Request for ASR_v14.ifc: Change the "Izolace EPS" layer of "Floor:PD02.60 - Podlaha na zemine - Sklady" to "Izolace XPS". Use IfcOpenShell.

First a look at what the model holds.

```python
import ifcopenshell
import ifcopenshell.util.element

model = ifcopenshell.open("ASR_v14.ifc")
print(model.schema)
for layer_set in model.by_type("IfcMaterialLayerSet"):
    if layer_set.LayerSetName == "Floor:PD02.60 - Podlaha na zemine - Sklady":
        for layer in layer_set.MaterialLayers:
            print(layer.id(), layer.Material and layer.Material.Name, layer.LayerThickness, sep=" | ")
        print(len(ifcopenshell.util.element.get_elements_by_material(model, layer_set)), "elements and types use it")
print(sorted(m.Name for m in model.by_type("IfcMaterial") if m.Name)[:60])
```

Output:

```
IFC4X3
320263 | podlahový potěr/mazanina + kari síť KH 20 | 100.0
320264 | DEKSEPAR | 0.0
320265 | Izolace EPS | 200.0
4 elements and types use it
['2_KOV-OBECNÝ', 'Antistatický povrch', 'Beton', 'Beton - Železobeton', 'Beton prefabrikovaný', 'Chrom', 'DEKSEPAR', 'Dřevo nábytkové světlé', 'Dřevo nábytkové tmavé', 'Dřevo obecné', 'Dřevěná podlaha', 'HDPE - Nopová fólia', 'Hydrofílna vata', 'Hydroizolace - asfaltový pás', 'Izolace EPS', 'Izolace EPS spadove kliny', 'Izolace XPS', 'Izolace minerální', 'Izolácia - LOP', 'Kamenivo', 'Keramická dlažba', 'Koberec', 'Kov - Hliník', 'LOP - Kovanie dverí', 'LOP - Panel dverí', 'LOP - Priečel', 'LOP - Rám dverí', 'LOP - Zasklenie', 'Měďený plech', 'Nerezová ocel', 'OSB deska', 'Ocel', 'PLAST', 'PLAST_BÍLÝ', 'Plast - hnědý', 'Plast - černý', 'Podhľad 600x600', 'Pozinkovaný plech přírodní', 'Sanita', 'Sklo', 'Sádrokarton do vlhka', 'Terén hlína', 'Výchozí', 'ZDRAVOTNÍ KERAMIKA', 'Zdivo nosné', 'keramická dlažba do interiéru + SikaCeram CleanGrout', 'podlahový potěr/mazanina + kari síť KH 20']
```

```python
import ifcopenshell
import ifcopenshell.api.material

model = ifcopenshell.open("ASR_v14.ifc")

layer_set = next(s for s in model.by_type("IfcMaterialLayerSet") if s.LayerSetName == "Floor:PD02.60 - Podlaha na zemine - Sklady")
layer = next(l for l in layer_set.MaterialLayers if l.Material and l.Material.Name == "Izolace EPS")
material = next(m for m in model.by_type("IfcMaterial") if m.Name == "Izolace XPS")

# Point this one layer at the other material; renaming the old one would change it everywhere.
ifcopenshell.api.material.edit_layer(model, layer=layer, attributes={"Name": material.Name}, material=material)

print([l.Material.Name if l.Material else None for l in layer_set.MaterialLayers])

model.write("ASR_v14_v2.ifc")
```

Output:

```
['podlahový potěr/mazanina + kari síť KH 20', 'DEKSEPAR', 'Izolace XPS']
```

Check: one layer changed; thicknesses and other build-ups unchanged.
